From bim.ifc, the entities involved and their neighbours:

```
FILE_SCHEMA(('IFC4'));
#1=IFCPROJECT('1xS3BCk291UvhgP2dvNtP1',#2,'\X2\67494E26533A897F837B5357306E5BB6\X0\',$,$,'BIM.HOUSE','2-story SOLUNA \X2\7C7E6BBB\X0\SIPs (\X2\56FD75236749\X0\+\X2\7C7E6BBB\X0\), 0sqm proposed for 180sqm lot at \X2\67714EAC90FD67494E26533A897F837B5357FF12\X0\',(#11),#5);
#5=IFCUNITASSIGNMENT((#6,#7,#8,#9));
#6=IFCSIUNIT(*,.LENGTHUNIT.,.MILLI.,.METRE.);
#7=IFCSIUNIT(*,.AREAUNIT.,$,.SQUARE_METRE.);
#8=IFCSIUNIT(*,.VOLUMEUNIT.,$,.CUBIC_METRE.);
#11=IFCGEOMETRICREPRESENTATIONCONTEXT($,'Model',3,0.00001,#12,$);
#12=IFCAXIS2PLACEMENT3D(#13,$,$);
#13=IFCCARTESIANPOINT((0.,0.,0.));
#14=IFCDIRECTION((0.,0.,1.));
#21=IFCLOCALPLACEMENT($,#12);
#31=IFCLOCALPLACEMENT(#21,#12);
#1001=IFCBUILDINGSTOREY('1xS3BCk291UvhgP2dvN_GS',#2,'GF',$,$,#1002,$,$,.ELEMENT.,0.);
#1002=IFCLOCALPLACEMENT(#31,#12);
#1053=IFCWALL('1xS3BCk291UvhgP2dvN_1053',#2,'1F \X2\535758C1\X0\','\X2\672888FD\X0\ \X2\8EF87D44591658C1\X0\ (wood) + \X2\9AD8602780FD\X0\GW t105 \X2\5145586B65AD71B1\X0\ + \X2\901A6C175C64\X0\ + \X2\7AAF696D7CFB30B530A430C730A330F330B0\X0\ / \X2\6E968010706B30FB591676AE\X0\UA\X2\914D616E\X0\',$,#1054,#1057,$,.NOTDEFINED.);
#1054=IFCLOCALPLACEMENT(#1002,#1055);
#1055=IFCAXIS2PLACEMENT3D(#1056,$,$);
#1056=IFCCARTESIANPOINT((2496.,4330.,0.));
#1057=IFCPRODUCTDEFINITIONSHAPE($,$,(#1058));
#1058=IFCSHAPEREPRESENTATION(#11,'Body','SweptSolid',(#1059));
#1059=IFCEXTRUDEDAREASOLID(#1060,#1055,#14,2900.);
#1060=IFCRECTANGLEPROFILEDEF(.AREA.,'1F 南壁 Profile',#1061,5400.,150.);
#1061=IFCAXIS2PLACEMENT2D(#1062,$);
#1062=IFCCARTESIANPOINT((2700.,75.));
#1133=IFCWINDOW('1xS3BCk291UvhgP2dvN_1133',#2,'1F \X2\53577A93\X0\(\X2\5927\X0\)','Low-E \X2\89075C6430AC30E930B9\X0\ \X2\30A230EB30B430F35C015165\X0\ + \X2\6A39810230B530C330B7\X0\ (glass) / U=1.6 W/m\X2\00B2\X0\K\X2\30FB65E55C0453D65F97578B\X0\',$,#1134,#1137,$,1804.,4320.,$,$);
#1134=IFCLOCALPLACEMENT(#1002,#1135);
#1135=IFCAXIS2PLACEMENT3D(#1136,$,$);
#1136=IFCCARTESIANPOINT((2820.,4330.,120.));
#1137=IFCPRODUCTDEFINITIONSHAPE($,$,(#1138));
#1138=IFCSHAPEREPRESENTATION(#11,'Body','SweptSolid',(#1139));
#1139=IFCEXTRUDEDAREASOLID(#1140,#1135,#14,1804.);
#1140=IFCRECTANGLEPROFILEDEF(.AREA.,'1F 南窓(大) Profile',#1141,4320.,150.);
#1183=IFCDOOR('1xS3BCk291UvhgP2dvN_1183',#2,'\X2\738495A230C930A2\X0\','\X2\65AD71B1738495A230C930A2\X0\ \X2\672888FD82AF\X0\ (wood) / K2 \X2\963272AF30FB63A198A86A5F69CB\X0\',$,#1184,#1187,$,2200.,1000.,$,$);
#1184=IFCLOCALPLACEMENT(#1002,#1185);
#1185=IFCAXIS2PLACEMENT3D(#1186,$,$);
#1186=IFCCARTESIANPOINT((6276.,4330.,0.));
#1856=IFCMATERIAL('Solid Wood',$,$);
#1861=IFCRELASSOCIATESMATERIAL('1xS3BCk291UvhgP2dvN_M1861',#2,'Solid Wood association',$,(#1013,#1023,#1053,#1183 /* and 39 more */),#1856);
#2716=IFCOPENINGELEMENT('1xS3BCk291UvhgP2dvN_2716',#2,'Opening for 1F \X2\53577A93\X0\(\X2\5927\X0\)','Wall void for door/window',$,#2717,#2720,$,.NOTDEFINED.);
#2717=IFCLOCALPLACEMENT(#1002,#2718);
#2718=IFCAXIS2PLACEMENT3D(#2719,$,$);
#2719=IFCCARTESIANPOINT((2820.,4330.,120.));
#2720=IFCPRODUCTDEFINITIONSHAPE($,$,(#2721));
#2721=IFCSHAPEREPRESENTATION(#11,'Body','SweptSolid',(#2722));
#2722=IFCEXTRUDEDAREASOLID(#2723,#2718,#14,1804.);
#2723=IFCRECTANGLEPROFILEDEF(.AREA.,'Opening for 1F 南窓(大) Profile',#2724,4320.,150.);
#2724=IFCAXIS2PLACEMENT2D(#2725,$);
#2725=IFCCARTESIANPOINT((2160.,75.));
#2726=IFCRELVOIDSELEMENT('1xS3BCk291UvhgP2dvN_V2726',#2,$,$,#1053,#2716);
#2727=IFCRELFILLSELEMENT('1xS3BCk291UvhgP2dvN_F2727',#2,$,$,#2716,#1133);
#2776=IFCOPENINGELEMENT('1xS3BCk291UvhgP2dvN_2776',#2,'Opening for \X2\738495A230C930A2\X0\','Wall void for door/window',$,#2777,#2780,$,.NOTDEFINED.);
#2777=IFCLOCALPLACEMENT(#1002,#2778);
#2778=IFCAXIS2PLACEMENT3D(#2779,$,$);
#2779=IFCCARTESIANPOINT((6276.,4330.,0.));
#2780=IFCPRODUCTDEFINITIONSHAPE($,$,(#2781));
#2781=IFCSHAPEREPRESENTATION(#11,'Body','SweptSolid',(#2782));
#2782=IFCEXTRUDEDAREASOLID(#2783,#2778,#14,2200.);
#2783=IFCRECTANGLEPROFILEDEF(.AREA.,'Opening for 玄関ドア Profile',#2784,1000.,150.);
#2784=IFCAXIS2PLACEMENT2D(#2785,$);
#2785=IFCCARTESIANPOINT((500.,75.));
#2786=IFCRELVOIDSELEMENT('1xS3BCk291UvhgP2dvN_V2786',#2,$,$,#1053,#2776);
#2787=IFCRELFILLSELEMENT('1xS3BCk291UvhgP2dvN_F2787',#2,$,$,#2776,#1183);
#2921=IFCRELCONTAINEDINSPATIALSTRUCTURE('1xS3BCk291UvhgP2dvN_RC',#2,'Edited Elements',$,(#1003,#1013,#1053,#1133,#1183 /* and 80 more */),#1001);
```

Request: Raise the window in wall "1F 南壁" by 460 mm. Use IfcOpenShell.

```python
import numpy as np
import ifcopenshell
import ifcopenshell.api.geometry
import ifcopenshell.util.placement
import ifcopenshell.util.unit

model = ifcopenshell.open("bim.ifc")
unit_scale = ifcopenshell.util.unit.calculate_unit_scale(model)

window = model.by_id(1133)
opening = window.FillsVoids[0].RelatingOpeningElement
dz = 0.46 / unit_scale

shift = np.array([0.0, 0.0, dz])
# The window is not placed relative to its opening, so move both.
for product in (opening, window):
    matrix = ifcopenshell.util.placement.get_local_placement(product.ObjectPlacement)
    matrix[:3, 3] += shift
    ifcopenshell.api.geometry.edit_object_placement(model, product=product, matrix=matrix, is_si=False)

print(f"moved by {dz * unit_scale:+.3f} m")

model.write("bim-out.ifc")
```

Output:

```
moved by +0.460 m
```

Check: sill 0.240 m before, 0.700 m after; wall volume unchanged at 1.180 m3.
